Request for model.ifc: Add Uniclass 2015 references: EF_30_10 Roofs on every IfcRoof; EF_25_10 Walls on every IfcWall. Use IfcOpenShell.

First a look at what the model holds.

```python
import ifcopenshell

model = ifcopenshell.open("model.ifc")
print(model.schema)
print("classifications:", [c.Name for c in model.by_type("IfcClassification")])
for ifc_class in ("IfcDoor", "IfcRoof", "IfcStair", "IfcWall", "IfcWindow"):
    print(ifc_class, len(model.by_type(ifc_class)))
```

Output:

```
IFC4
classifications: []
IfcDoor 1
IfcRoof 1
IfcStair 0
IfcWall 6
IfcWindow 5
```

```python
import ifcopenshell
import ifcopenshell.api.classification

model = ifcopenshell.open("model.ifc")

system = ifcopenshell.api.classification.add_classification(model, classification="Uniclass 2015")

codes = {
    "IfcRoof": ("EF_30_10", "Roofs"),
    "IfcWall": ("EF_25_10", "Walls"),
}
for ifc_class, (code, name) in codes.items():
    products = model.by_type(ifc_class)
    ifcopenshell.api.classification.add_reference(
        model, products=products, classification=system, identification=code, name=name
    )
    print(code, len(products))

model.write("model-out.ifc")
```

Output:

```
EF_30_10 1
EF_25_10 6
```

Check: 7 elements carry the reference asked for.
